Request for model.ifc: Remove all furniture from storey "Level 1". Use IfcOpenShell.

First a look at what the model holds.

```python
import ifcopenshell
import ifcopenshell.util.element

model = ifcopenshell.open("model.ifc")
print(model.schema)
storey = next(s for s in model.by_type("IfcBuildingStorey") if s.Name == "Level 1")
furniture = [e for e in ifcopenshell.util.element.get_decomposition(storey) if e.is_a("IfcFurnishingElement")]
seen = {}
for e in furniture:
    element_type = ifcopenshell.util.element.get_type(e)
    name = element_type.Name if element_type not in (None, e) else None
    seen[name] = seen.get(name, 0) + 1
for name, count in sorted(seen.items(), key=str):
    print(count, "x", name)
```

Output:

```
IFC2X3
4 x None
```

```python
import ifcopenshell
import ifcopenshell.api.root
import ifcopenshell.util.element

model = ifcopenshell.open("model.ifc")

storey = next(s for s in model.by_type("IfcBuildingStorey") if s.Name == "Level 1")
furniture = [e for e in ifcopenshell.util.element.get_decomposition(storey) if e.is_a("IfcFurnishingElement")]

for e in furniture:
    ifcopenshell.api.root.remove_product(model, product=e)
print(len(furniture), "removed")

model.write("model_edited.ifc")
```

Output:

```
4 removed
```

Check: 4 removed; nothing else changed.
